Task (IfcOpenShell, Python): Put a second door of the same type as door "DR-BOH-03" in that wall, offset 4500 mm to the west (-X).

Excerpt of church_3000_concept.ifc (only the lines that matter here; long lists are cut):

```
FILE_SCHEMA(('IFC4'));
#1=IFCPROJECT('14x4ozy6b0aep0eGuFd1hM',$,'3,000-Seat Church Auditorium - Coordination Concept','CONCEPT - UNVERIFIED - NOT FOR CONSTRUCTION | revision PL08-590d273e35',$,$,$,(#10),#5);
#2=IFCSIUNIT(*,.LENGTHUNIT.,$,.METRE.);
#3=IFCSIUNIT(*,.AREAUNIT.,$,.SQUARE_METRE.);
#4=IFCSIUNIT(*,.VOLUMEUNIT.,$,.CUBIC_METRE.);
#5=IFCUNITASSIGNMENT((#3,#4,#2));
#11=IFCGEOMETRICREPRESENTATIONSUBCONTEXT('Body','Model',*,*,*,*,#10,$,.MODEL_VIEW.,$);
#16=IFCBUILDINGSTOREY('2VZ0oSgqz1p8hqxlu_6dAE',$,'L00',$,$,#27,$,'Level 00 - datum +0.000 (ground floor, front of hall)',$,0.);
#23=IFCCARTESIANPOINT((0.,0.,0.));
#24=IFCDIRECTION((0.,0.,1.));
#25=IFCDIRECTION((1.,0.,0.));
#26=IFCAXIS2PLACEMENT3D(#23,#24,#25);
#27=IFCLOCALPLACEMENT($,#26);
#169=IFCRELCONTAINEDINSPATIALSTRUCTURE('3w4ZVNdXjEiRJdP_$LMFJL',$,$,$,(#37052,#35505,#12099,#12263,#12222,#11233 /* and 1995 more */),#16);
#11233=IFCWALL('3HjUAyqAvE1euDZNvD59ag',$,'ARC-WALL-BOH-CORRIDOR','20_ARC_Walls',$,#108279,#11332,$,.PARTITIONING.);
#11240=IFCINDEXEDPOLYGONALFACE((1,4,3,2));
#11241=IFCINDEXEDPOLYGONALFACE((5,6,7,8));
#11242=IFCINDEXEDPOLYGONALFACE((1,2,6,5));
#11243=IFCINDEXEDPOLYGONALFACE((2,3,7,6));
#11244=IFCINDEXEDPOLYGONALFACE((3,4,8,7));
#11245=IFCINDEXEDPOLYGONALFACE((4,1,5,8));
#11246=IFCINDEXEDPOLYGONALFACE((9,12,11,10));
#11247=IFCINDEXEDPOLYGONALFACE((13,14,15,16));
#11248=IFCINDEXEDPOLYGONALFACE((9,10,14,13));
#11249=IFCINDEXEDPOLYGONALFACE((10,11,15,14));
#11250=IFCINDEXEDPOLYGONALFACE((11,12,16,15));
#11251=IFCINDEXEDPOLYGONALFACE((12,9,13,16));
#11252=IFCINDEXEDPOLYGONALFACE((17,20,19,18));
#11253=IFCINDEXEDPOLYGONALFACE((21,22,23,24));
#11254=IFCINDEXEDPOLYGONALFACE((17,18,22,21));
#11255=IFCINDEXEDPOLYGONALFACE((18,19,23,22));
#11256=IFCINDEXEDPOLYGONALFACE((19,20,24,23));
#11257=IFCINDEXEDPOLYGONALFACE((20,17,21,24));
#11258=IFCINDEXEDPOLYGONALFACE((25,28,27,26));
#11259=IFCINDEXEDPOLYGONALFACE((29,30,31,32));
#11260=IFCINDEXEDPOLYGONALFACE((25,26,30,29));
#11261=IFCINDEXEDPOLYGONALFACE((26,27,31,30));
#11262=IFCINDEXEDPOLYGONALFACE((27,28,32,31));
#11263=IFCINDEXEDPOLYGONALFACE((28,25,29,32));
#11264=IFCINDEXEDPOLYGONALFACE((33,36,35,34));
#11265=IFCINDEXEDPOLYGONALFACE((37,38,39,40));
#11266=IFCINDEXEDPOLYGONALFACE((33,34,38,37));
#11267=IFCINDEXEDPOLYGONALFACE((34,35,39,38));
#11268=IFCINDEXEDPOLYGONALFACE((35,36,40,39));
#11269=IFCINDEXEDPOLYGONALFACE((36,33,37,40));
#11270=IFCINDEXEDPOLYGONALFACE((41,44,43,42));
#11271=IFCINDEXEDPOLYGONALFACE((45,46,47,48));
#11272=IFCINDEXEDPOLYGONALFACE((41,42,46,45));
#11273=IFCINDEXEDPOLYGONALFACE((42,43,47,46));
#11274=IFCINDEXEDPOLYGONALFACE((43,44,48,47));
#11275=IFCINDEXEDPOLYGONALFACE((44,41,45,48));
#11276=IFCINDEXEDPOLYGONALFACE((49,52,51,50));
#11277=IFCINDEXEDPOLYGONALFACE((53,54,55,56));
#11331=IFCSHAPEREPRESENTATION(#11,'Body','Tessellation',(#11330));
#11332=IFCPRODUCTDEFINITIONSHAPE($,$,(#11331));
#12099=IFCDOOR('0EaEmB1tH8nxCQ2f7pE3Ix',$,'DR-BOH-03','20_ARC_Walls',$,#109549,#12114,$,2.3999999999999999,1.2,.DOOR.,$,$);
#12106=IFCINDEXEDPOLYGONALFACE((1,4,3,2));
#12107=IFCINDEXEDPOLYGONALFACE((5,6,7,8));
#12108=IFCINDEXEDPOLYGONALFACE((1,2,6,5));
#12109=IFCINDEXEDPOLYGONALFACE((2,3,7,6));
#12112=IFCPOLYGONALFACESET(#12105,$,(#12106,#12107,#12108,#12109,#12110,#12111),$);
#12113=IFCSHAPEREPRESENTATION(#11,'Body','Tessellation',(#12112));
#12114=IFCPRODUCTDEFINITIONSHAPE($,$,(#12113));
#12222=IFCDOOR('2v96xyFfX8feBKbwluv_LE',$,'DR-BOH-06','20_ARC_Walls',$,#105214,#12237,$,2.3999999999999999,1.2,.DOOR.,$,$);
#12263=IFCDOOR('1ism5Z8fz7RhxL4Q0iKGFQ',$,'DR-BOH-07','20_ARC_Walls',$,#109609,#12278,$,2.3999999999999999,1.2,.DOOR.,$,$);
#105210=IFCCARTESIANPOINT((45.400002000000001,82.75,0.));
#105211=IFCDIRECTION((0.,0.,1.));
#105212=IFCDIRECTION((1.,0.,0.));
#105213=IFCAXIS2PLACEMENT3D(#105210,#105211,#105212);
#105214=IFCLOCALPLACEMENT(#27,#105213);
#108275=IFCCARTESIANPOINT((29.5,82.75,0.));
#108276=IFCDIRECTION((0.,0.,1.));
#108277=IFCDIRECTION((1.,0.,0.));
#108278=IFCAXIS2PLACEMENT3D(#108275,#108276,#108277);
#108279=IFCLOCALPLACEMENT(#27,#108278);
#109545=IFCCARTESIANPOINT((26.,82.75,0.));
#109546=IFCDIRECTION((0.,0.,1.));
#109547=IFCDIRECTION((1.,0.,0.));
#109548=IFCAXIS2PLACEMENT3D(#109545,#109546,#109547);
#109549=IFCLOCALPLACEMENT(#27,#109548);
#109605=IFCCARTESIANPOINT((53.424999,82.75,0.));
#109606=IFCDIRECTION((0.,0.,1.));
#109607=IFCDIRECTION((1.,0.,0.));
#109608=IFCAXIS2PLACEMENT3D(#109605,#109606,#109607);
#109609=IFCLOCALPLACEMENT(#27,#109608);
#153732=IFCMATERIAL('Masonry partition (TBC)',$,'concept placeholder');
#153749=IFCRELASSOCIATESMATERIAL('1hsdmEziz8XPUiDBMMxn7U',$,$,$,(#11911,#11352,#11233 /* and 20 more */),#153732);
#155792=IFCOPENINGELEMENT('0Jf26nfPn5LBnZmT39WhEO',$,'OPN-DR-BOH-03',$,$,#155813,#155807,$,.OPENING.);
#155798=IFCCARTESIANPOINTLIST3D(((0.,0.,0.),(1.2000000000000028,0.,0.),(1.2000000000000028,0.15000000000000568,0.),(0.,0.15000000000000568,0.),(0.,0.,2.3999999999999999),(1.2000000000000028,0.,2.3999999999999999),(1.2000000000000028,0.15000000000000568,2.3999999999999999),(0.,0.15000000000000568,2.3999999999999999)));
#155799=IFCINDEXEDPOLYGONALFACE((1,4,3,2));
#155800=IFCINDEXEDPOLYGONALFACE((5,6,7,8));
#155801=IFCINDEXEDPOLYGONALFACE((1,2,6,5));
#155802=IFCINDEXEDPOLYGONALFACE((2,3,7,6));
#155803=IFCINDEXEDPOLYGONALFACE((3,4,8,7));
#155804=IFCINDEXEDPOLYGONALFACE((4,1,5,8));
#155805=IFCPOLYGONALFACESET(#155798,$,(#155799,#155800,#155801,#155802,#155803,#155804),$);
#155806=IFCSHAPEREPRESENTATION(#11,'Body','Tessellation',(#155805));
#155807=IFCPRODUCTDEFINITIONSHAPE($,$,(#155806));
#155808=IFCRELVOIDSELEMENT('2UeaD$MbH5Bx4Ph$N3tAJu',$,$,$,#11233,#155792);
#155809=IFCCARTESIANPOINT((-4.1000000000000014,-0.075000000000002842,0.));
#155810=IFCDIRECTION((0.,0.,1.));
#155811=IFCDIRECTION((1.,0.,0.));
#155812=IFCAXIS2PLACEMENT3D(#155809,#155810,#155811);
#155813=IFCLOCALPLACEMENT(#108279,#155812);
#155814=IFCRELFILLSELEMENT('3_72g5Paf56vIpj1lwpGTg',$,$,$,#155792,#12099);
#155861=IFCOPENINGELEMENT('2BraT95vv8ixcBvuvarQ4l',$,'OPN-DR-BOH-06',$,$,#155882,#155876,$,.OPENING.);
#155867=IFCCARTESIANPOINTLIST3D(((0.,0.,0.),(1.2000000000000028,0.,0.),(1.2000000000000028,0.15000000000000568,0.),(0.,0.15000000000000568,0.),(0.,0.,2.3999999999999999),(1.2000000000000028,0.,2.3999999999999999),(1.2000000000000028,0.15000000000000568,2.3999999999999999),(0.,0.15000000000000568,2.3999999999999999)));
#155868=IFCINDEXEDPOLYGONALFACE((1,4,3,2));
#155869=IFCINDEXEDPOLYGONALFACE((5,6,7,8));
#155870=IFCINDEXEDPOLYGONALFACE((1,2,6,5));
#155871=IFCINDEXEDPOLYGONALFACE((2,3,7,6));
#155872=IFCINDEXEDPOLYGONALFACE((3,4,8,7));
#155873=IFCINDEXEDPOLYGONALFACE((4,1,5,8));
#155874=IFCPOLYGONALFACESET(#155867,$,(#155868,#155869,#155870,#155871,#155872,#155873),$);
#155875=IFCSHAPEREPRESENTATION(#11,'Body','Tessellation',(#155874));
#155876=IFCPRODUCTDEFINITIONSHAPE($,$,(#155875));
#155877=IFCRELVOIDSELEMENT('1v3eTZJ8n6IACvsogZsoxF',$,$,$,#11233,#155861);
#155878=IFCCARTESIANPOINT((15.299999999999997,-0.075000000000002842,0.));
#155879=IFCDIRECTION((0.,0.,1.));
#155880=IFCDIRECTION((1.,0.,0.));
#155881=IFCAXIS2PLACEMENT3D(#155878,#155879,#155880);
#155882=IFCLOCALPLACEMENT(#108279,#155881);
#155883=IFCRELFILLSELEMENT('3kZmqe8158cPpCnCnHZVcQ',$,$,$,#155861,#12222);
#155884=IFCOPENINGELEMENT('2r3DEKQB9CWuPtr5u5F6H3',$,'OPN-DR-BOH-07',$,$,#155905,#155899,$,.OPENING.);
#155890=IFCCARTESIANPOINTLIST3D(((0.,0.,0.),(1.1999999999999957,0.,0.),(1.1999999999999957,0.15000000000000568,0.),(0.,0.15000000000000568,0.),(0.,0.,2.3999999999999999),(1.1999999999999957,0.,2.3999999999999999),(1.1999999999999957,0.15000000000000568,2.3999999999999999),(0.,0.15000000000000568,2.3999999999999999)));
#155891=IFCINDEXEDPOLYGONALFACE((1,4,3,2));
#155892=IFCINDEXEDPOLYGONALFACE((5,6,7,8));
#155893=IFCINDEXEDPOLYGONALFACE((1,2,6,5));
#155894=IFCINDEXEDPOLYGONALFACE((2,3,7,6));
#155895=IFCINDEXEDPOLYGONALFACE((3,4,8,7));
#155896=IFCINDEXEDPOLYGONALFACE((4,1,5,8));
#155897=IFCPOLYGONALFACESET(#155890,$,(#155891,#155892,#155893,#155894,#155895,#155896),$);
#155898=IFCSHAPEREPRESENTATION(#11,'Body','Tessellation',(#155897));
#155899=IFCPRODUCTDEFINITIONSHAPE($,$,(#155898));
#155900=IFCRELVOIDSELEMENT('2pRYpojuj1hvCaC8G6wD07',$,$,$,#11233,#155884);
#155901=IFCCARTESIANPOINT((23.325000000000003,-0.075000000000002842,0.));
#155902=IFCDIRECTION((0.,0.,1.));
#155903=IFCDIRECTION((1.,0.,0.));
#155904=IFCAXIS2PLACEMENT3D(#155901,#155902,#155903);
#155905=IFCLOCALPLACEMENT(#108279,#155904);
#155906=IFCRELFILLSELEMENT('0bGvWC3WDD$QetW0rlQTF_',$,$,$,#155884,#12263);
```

```python
import ifcopenshell
import ifcopenshell.api.feature
import ifcopenshell.api.geometry
import ifcopenshell.api.root
import ifcopenshell.geom
import ifcopenshell.util.element
import ifcopenshell.util.placement
import ifcopenshell.util.shape
import ifcopenshell.util.unit

model = ifcopenshell.open("church_3000_concept.ifc")
unit_scale = ifcopenshell.util.unit.calculate_unit_scale(model)
settings = ifcopenshell.geom.settings()


def volume(element):
    """Net volume in cubic metres, openings subtracted."""
    shape = ifcopenshell.geom.create_shape(settings, element)
    return ifcopenshell.util.shape.get_volume(shape.geometry)


door = model.by_guid("0EaEmB1tH8nxCQ2f7pE3Ix")
opening = door.FillsVoids[0].RelatingOpeningElement
wall = opening.VoidsElements[0].RelatingBuildingElement
before = volume(wall)
shift = ifcopenshell.util.placement.get_local_placement(wall.ObjectPlacement)[:3, 0] * -4.5 / unit_scale

# copy_class copies the void relationship, type, container and properties, but no geometry.
new_opening = ifcopenshell.api.root.copy_class(model, product=opening)
new_opening.Representation = ifcopenshell.util.element.copy_deep(
    model, opening.Representation, exclude=["IfcGeometricRepresentationContext", "IfcRepresentationMap"]
)
new_door = ifcopenshell.api.root.copy_class(model, product=door)
new_door.Representation = ifcopenshell.util.element.copy_deep(
    model, door.Representation, exclude=["IfcGeometricRepresentationContext", "IfcRepresentationMap"]
)
ifcopenshell.api.feature.add_filling(model, opening=new_opening, element=new_door)

for old, new in ((opening, new_opening), (door, new_door)):
    matrix = ifcopenshell.util.placement.get_local_placement(old.ObjectPlacement)
    matrix[:3, 3] += shift
    ifcopenshell.api.geometry.edit_object_placement(model, product=new, matrix=matrix, is_si=False)

after = volume(wall)

print(f"wall volume {before:.3f} -> {after:.3f} m3")

model.write("church_3000_concept-out.ifc")
```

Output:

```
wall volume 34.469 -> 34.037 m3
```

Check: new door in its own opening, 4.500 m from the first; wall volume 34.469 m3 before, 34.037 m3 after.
